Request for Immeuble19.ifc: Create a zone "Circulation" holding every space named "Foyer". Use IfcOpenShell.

First a look at what the model holds.

```python
import ifcopenshell

model = ifcopenshell.open("Immeuble19.ifc")
print(model.schema)
seen = {}
for space in model.by_type("IfcSpace"):
    seen[space.LongName] = seen.get(space.LongName, 0) + 1
for name, count in sorted(seen.items(), key=str):
    print(count, "x", name)
print("zones:", [z.Name for z in model.by_type("IfcZone")][:20])
```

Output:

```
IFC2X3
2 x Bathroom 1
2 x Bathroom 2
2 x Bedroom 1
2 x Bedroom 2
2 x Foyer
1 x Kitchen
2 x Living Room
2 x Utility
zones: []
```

```python
import ifcopenshell
import ifcopenshell.api.group
import ifcopenshell.api.root

model = ifcopenshell.open("Immeuble19.ifc")

names = {"Foyer"}
spaces = [s for s in model.by_type("IfcSpace") if s.LongName in names]

zone = ifcopenshell.api.root.create_entity(model, ifc_class="IfcZone", name="Circulation")
ifcopenshell.api.group.assign_group(model, products=spaces, group=zone)
print(len(spaces), "spaces in", zone.Name)

model.write("Immeuble19_updated.ifc")
```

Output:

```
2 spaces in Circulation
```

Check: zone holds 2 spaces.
